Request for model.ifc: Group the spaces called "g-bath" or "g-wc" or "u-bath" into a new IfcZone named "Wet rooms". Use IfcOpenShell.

First a look at what the model holds.

```python
import ifcopenshell

model = ifcopenshell.open("model.ifc")
print(model.schema)
seen = {}
for space in model.by_type("IfcSpace"):
    seen[space.LongName] = seen.get(space.LongName, 0) + 1
for name, count in sorted(seen.items(), key=str):
    print(count, "x", name)
print("zones:", [z.Name for z in model.by_type("IfcZone")][:20])
```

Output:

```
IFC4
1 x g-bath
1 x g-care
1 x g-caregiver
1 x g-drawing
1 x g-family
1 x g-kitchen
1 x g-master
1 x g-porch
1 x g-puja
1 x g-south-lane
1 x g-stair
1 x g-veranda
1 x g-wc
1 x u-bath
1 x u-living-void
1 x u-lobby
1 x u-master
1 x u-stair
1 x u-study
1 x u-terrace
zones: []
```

```python
import ifcopenshell
import ifcopenshell.api.group
import ifcopenshell.api.root

model = ifcopenshell.open("model.ifc")

names = {"g-bath", "g-wc", "u-bath"}
spaces = [s for s in model.by_type("IfcSpace") if s.LongName in names]

zone = ifcopenshell.api.root.create_entity(model, ifc_class="IfcZone", name="Wet rooms")
ifcopenshell.api.group.assign_group(model, products=spaces, group=zone)
print(len(spaces), "spaces in", zone.Name)

model.write("model-out.ifc")
```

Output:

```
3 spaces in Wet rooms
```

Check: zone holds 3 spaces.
